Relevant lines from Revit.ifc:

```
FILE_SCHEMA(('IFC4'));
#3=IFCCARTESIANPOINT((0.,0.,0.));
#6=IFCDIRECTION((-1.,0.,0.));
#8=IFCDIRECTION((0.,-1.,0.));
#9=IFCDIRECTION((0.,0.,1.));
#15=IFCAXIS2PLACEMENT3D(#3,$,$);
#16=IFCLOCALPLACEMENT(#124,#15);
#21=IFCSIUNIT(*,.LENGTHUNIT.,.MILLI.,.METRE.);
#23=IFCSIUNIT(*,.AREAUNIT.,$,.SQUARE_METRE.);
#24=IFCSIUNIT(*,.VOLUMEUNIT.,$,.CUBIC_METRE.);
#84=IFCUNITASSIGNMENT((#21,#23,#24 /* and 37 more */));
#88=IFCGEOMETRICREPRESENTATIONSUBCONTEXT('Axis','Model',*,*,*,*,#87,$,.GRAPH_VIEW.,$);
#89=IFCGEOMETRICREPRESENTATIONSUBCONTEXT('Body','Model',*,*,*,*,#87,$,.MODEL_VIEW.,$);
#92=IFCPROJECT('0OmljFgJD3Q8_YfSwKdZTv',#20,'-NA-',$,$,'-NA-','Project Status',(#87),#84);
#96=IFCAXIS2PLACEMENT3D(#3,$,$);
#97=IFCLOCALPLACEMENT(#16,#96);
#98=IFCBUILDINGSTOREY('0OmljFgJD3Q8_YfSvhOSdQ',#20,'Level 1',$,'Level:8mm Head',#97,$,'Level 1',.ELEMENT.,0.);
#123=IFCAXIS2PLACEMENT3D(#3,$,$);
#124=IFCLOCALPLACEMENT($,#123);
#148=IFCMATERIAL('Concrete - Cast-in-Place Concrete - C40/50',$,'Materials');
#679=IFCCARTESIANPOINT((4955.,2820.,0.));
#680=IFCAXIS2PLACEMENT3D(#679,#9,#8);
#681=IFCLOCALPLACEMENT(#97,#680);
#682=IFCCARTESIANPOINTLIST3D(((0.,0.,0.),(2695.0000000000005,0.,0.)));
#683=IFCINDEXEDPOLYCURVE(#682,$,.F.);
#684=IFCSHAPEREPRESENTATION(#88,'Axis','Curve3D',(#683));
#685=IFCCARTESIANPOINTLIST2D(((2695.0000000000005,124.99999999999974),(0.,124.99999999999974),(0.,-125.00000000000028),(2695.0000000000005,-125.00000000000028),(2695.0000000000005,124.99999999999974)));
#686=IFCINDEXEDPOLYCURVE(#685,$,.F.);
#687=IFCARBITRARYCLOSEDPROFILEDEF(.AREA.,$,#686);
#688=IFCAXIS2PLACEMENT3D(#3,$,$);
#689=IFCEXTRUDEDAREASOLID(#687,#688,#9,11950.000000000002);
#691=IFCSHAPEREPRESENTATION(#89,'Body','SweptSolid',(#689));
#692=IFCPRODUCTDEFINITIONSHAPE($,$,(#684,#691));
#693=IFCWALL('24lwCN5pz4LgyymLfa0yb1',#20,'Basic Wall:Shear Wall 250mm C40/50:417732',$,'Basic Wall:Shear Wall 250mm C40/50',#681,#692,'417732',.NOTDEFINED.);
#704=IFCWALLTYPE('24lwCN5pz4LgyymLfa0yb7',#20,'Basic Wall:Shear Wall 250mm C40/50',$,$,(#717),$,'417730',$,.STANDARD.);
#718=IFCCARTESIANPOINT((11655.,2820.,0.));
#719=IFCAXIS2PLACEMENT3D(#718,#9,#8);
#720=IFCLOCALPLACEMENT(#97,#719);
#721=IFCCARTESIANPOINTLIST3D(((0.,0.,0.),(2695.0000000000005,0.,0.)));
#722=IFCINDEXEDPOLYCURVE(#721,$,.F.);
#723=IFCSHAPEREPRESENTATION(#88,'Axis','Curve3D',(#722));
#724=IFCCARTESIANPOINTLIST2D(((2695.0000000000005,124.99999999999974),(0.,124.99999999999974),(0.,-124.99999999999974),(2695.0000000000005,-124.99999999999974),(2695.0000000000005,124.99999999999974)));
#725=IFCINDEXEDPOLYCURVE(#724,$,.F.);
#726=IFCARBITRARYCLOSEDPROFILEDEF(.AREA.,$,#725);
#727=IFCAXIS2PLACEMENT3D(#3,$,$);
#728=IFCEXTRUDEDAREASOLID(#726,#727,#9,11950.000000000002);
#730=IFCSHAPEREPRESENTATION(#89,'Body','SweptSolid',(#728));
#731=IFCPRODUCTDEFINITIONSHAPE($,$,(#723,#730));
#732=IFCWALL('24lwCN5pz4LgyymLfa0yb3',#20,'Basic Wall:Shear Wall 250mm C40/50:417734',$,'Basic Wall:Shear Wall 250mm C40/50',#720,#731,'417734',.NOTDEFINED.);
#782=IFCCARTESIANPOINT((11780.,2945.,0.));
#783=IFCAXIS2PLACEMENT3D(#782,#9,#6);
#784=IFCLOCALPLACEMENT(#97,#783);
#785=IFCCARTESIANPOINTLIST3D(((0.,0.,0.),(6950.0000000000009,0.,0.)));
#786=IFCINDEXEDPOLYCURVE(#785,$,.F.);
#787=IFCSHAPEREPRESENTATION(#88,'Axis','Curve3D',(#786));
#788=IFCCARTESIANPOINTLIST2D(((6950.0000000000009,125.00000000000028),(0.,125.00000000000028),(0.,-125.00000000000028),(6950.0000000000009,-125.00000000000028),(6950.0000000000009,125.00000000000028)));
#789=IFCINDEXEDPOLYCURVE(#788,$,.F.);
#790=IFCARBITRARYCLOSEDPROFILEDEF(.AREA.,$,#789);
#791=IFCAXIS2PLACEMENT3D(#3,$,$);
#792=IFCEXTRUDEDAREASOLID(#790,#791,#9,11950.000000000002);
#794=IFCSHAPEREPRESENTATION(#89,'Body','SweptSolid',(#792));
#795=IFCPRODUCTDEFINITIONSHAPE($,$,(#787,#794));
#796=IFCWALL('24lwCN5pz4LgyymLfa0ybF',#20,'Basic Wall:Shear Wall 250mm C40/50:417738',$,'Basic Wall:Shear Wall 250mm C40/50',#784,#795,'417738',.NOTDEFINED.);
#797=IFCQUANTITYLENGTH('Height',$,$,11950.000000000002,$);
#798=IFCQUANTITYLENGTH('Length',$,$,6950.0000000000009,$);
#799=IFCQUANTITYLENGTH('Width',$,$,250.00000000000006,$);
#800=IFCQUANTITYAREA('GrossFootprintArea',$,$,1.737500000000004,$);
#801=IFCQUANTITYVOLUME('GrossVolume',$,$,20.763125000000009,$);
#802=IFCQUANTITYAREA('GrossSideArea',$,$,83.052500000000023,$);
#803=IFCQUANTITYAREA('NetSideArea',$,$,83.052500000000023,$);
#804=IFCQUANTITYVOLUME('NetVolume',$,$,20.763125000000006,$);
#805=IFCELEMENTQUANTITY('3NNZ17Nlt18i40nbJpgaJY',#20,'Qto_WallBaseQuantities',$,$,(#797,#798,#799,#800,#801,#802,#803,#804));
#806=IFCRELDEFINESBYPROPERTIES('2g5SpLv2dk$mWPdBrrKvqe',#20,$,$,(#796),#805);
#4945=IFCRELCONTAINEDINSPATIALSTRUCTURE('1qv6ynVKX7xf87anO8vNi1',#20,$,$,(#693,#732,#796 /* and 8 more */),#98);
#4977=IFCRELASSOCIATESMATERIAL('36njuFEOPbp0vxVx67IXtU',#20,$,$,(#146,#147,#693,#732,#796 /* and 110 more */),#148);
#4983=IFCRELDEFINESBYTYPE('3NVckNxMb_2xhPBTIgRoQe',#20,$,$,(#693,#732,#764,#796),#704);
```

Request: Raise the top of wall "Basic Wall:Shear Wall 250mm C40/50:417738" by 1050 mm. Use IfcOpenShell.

```python
import ifcopenshell
import ifcopenshell.api.pset
import ifcopenshell.geom
import ifcopenshell.util.element
import ifcopenshell.util.representation
import ifcopenshell.util.shape
import ifcopenshell.util.unit

model = ifcopenshell.open("Revit.ifc")
unit_scale = ifcopenshell.util.unit.calculate_unit_scale(model)
area_scale = ifcopenshell.util.unit.calculate_unit_scale(model, "AREAUNIT")
volume_scale = ifcopenshell.util.unit.calculate_unit_scale(model, "VOLUMEUNIT")
settings = ifcopenshell.geom.settings()


def volume(element):
    """Net volume in cubic metres, openings subtracted."""
    shape = ifcopenshell.geom.create_shape(settings, element)
    return ifcopenshell.util.shape.get_volume(shape.geometry)


wall = model.by_guid("24lwCN5pz4LgyymLfa0ybF")
before = volume(wall)

body = ifcopenshell.util.representation.get_representation(wall, "Model", "Body")
solid = body.Items[0]
old_height = solid.Depth
solid.Depth += 1050.0
after = volume(wall)
thickness = 0.25  # wall thickness in metres

# Update the stored height, areas and volumes.
qto = model.by_id(ifcopenshell.util.element.get_pset(wall, "Qto_WallBaseQuantities", should_inherit=False)["id"])
ifcopenshell.api.pset.edit_qto(model, qto=qto, properties={
    "Height": solid.Depth,
    "GrossVolume": ifcopenshell.util.element.get_pset(wall, "Qto_WallBaseQuantities", "GrossVolume") * solid.Depth / old_height,
    "GrossSideArea": ifcopenshell.util.element.get_pset(wall, "Qto_WallBaseQuantities", "GrossSideArea") * solid.Depth / old_height,
    "NetSideArea": after / thickness / area_scale,
    "NetVolume": after / volume_scale,
})

print(f"height {old_height:g} -> {solid.Depth:g}, volume {before:.3f} -> {after:.3f} m3")

model.write("Revit-out.ifc")
```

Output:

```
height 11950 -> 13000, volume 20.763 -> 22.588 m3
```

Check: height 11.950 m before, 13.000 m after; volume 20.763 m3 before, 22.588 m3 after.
